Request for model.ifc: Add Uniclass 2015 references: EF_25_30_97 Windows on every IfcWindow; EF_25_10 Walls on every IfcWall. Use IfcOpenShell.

First a look at what the model holds.

```python
import ifcopenshell

model = ifcopenshell.open("model.ifc")
print(model.schema)
print("classifications:", [c.Name for c in model.by_type("IfcClassification")])
for ifc_class in ("IfcDoor", "IfcRoof", "IfcStair", "IfcWall", "IfcWindow"):
    print(ifc_class, len(model.by_type(ifc_class)))
```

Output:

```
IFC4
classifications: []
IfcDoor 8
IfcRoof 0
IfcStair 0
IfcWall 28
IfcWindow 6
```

```python
import ifcopenshell
import ifcopenshell.api.classification

model = ifcopenshell.open("model.ifc")

system = ifcopenshell.api.classification.add_classification(model, classification="Uniclass 2015")

codes = {
    "IfcWindow": ("EF_25_30_97", "Windows"),
    "IfcWall": ("EF_25_10", "Walls"),
}
for ifc_class, (code, name) in codes.items():
    products = model.by_type(ifc_class)
    ifcopenshell.api.classification.add_reference(
        model, products=products, classification=system, identification=code, name=name
    )
    print(code, len(products))

model.write("model-out.ifc")
```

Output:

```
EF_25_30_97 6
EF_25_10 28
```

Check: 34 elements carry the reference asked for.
